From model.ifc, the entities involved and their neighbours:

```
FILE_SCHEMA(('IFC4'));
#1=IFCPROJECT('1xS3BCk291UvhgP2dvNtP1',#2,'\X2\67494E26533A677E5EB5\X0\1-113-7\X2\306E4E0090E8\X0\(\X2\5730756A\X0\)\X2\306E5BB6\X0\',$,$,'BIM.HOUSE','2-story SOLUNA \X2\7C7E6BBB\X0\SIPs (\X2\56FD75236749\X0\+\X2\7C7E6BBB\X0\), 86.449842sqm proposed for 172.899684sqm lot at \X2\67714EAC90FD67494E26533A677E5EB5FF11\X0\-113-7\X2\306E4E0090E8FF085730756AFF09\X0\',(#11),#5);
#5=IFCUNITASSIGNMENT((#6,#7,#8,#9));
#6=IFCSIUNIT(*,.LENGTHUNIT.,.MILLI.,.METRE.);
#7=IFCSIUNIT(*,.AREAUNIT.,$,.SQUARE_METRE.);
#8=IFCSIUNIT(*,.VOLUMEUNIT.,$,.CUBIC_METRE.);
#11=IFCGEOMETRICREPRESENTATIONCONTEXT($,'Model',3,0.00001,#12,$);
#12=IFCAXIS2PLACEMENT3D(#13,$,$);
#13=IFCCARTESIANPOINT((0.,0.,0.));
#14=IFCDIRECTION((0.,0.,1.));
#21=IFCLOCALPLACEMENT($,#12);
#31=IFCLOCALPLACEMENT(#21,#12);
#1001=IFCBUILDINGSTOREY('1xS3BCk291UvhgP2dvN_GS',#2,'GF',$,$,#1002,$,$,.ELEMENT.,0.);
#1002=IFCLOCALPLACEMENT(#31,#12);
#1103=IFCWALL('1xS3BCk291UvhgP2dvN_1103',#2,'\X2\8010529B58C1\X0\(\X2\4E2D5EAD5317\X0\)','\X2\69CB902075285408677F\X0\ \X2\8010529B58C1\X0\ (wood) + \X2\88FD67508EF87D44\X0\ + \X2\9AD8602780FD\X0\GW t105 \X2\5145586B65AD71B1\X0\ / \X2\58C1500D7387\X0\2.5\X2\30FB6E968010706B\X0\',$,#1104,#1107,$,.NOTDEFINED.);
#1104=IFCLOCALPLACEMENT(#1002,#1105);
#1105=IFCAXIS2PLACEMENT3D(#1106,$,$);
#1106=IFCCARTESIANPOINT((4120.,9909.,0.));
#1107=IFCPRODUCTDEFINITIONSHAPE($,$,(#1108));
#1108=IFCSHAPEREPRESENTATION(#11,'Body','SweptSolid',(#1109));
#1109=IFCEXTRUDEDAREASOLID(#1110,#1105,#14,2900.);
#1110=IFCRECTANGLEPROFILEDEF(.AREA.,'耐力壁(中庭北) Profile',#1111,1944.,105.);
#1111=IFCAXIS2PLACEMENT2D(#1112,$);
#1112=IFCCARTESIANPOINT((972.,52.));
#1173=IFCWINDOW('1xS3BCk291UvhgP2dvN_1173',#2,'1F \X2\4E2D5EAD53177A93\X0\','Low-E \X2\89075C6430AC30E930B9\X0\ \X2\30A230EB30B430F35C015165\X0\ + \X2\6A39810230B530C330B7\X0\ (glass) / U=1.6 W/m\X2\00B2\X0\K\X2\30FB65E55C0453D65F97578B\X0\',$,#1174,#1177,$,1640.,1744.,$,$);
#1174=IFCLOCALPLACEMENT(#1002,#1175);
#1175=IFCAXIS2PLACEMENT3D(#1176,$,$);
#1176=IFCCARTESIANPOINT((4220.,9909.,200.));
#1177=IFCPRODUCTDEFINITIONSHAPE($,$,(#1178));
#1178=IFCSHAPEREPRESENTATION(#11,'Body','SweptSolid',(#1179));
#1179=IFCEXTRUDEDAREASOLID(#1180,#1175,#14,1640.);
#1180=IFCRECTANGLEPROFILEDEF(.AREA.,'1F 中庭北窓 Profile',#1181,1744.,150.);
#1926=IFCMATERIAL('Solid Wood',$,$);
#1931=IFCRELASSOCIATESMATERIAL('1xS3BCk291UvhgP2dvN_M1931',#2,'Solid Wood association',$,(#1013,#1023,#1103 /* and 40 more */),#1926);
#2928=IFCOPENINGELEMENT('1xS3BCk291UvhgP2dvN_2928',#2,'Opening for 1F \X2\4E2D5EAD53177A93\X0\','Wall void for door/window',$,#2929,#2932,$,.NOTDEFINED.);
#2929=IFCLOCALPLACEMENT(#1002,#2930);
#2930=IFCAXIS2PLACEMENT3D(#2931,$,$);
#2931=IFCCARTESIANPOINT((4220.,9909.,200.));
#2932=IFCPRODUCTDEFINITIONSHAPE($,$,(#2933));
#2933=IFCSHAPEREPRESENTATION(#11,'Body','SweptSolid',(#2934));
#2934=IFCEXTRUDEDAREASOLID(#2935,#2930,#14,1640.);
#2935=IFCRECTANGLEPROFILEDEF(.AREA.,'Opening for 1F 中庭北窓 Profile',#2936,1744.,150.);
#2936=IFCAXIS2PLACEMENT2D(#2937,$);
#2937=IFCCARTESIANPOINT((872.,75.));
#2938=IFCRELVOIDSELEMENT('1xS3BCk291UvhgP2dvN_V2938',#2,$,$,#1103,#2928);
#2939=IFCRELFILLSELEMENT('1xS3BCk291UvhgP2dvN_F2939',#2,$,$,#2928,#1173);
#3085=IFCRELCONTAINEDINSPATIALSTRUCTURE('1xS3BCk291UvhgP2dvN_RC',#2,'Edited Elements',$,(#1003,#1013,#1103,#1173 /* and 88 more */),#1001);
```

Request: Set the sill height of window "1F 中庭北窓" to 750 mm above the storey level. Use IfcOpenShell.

```python
import numpy as np
import ifcopenshell
import ifcopenshell.api.geometry
import ifcopenshell.geom
import ifcopenshell.util.element
import ifcopenshell.util.placement
import ifcopenshell.util.shape
import ifcopenshell.util.unit

model = ifcopenshell.open("model.ifc")
unit_scale = ifcopenshell.util.unit.calculate_unit_scale(model)

window = model.by_id(1173)
opening = window.FillsVoids[0].RelatingOpeningElement
storey = ifcopenshell.util.element.get_container(window, ifc_class="IfcBuildingStorey")
level = ifcopenshell.util.placement.get_local_placement(storey.ObjectPlacement)[2, 3]

# The opening's origin need not be at the sill, so measure its lowest point.
shape = ifcopenshell.geom.create_shape(ifcopenshell.geom.settings(), opening)
bottom = ifcopenshell.util.shape.get_shape_bottom_elevation(shape, shape.geometry) / unit_scale
dz = level + 750.0 - bottom

shift = np.array([0.0, 0.0, dz])
# The window is not placed relative to its opening, so move both.
for product in (opening, window):
    matrix = ifcopenshell.util.placement.get_local_placement(product.ObjectPlacement)
    matrix[:3, 3] += shift
    ifcopenshell.api.geometry.edit_object_placement(model, product=product, matrix=matrix, is_si=False)

print(f"moved by {dz * unit_scale:+.3f} m")

model.write("model_v2.ifc")
```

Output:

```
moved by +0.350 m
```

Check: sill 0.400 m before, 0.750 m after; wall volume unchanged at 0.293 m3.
